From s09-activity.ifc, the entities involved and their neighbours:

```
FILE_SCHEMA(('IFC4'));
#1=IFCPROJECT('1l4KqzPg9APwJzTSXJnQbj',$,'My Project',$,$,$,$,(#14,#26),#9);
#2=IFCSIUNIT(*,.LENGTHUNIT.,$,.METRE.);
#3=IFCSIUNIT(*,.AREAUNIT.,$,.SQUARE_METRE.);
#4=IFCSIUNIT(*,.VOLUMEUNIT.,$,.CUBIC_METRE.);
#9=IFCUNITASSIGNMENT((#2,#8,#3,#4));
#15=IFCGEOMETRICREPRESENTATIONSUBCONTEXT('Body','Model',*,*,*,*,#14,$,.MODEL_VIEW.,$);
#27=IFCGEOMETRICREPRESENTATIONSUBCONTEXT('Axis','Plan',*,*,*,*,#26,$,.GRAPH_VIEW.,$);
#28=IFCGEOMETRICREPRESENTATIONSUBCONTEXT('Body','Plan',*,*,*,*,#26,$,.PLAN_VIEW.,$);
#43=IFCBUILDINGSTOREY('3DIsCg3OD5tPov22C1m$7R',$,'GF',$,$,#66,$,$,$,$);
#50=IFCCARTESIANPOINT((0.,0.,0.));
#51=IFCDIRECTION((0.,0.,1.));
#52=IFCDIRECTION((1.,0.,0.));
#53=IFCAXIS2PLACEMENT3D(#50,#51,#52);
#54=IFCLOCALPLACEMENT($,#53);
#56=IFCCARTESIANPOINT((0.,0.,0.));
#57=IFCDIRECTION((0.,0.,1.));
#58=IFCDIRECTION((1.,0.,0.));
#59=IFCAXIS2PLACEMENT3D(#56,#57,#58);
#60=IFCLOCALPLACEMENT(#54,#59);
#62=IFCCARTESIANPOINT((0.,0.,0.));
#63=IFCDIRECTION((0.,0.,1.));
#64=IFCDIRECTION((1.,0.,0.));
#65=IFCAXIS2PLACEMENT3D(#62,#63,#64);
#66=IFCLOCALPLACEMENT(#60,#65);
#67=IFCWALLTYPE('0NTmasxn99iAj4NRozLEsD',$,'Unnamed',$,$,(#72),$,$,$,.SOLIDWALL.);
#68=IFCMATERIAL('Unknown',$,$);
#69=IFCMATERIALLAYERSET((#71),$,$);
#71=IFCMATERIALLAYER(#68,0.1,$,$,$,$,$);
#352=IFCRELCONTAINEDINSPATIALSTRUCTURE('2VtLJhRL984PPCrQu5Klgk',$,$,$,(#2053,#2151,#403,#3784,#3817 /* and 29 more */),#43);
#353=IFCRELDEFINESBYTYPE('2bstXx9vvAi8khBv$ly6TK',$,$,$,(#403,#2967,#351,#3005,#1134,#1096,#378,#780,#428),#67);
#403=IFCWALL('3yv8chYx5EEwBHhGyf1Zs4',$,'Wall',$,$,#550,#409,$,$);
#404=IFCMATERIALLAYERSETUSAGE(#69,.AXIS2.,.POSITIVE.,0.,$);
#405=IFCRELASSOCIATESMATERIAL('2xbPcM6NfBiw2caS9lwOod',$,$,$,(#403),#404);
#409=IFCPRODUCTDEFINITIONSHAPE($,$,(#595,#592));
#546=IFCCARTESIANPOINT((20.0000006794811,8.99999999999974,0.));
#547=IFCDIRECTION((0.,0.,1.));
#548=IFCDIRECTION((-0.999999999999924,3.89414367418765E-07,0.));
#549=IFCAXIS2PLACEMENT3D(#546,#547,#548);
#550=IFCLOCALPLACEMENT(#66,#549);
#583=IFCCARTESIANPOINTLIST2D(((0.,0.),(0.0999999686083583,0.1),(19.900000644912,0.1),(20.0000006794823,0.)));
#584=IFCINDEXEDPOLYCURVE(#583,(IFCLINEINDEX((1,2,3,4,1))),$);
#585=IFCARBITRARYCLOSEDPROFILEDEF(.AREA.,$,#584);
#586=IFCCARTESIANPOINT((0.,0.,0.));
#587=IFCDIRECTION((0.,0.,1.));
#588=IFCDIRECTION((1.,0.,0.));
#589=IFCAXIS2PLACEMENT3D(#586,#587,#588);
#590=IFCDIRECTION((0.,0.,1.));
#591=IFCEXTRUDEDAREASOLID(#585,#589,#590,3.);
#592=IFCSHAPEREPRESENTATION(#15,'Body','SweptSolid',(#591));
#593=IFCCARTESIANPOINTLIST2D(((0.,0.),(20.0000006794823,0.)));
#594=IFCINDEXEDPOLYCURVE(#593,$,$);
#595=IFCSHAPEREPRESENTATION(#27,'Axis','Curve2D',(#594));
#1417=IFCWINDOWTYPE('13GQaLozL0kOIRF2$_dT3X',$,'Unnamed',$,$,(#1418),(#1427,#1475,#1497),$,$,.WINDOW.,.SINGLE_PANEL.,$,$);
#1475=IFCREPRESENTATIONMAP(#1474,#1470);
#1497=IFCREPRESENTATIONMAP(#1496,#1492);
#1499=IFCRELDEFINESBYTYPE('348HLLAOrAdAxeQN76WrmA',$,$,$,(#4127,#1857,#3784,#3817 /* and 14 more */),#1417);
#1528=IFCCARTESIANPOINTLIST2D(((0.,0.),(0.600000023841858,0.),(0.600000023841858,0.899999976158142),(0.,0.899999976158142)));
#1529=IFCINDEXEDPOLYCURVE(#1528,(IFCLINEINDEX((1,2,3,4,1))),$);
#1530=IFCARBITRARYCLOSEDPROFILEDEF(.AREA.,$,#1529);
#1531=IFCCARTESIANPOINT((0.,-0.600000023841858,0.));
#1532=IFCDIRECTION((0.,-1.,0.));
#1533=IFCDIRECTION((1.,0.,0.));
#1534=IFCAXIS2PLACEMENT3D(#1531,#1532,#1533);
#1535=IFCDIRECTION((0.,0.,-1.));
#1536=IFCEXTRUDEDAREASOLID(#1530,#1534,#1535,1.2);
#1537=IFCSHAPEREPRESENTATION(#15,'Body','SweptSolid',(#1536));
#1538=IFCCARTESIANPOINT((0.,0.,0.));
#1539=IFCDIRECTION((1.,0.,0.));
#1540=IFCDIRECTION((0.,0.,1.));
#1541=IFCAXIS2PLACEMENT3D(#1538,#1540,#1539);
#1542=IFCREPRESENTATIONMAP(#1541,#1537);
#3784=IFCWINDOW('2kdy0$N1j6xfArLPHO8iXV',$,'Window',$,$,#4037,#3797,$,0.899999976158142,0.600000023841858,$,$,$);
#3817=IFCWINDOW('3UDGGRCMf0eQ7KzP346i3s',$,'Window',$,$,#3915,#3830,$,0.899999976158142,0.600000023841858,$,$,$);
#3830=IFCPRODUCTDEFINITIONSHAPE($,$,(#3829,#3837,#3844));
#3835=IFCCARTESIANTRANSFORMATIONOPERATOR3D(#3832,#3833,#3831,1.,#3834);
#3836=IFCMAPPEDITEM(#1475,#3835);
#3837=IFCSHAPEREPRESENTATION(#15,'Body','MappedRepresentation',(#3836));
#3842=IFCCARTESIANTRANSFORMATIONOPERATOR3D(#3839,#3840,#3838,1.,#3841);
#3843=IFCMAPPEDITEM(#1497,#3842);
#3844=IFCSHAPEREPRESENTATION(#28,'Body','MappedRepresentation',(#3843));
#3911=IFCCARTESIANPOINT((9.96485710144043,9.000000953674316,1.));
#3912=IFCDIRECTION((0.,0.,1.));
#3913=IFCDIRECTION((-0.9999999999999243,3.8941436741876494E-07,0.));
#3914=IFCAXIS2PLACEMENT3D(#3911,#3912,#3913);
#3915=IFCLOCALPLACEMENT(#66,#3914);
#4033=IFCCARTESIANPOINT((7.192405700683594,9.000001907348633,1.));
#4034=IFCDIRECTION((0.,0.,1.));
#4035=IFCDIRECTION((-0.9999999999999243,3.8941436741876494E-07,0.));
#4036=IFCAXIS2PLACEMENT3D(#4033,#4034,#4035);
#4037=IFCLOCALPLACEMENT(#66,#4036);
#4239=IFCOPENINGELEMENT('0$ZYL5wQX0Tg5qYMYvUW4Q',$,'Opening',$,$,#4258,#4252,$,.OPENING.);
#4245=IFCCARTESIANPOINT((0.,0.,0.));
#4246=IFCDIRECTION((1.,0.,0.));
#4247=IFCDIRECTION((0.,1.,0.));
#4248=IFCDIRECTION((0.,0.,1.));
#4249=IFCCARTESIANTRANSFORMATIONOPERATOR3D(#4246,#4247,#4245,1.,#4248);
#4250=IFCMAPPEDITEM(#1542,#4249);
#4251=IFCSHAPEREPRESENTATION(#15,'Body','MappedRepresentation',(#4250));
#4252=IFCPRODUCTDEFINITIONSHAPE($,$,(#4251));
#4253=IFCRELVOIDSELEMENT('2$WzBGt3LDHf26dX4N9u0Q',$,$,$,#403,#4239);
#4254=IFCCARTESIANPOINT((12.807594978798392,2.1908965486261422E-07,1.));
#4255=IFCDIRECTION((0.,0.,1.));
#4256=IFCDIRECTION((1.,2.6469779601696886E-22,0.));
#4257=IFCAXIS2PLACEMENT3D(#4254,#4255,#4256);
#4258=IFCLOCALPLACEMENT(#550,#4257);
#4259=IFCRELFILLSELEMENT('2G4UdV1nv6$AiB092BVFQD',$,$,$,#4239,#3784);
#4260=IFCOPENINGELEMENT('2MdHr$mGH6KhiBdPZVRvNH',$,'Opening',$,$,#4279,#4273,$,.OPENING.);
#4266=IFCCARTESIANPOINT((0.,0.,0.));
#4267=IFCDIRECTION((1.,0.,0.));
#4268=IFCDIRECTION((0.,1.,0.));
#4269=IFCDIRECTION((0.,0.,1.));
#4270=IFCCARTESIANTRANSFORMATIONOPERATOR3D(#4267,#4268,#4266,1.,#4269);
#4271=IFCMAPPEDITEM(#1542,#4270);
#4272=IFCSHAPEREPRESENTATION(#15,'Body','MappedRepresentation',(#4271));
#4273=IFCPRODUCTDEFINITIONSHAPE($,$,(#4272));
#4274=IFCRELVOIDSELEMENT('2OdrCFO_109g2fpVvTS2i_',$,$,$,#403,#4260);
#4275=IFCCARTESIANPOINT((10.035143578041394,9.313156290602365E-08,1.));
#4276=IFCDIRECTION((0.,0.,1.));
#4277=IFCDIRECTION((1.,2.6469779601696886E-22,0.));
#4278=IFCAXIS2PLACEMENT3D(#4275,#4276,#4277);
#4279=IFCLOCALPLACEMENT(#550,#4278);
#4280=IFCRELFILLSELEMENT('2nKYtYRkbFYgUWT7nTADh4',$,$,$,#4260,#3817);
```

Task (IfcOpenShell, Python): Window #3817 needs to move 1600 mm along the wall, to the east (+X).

```python
import ifcopenshell
import ifcopenshell.api.geometry
import ifcopenshell.util.placement

model = ifcopenshell.open("s09-activity.ifc")

window = model.by_guid("3UDGGRCMf0eQ7KzP346i3s")
opening = window.FillsVoids[0].RelatingOpeningElement
wall = opening.VoidsElements[0].RelatingBuildingElement

wall_matrix = ifcopenshell.util.placement.get_local_placement(wall.ObjectPlacement)
shift = wall_matrix[:3, 0] * -1.6
before = ifcopenshell.util.placement.get_local_placement(window.ObjectPlacement)[:3, 3].copy()

# The window is not placed relative to its opening, so move both.
for product in (opening, window):
    matrix = ifcopenshell.util.placement.get_local_placement(product.ObjectPlacement)
    matrix[:3, 3] += shift
    ifcopenshell.api.geometry.edit_object_placement(model, product=product, matrix=matrix, is_si=False)

after = ifcopenshell.util.placement.get_local_placement(window.ObjectPlacement)[:3, 3]
print("window moved by", (after - before).round(3) + 0.0)

model.write("s09-activity_rev.ifc")
```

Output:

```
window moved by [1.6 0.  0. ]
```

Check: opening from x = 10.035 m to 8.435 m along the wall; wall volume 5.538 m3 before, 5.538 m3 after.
